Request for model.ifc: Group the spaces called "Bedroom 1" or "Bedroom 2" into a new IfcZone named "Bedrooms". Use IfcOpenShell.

First a look at what the model holds.

```python
import ifcopenshell

model = ifcopenshell.open("model.ifc")
print(model.schema)
seen = {}
for space in model.by_type("IfcSpace"):
    seen[space.LongName] = seen.get(space.LongName, 0) + 1
for name, count in sorted(seen.items(), key=str):
    print(count, "x", name)
print("zones:", [z.Name for z in model.by_type("IfcZone")][:20])
```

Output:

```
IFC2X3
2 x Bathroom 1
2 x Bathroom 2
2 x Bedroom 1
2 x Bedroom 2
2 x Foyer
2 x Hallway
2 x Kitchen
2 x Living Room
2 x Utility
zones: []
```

```python
import ifcopenshell
import ifcopenshell.api.group
import ifcopenshell.api.root

model = ifcopenshell.open("model.ifc")

names = {"Bedroom 1", "Bedroom 2"}
spaces = [s for s in model.by_type("IfcSpace") if s.LongName in names]

zone = ifcopenshell.api.root.create_entity(model, ifc_class="IfcZone", name="Bedrooms")
ifcopenshell.api.group.assign_group(model, products=spaces, group=zone)
print(len(spaces), "spaces in", zone.Name)

model.write("model_rev.ifc")
```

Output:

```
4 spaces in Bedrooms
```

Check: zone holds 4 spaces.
